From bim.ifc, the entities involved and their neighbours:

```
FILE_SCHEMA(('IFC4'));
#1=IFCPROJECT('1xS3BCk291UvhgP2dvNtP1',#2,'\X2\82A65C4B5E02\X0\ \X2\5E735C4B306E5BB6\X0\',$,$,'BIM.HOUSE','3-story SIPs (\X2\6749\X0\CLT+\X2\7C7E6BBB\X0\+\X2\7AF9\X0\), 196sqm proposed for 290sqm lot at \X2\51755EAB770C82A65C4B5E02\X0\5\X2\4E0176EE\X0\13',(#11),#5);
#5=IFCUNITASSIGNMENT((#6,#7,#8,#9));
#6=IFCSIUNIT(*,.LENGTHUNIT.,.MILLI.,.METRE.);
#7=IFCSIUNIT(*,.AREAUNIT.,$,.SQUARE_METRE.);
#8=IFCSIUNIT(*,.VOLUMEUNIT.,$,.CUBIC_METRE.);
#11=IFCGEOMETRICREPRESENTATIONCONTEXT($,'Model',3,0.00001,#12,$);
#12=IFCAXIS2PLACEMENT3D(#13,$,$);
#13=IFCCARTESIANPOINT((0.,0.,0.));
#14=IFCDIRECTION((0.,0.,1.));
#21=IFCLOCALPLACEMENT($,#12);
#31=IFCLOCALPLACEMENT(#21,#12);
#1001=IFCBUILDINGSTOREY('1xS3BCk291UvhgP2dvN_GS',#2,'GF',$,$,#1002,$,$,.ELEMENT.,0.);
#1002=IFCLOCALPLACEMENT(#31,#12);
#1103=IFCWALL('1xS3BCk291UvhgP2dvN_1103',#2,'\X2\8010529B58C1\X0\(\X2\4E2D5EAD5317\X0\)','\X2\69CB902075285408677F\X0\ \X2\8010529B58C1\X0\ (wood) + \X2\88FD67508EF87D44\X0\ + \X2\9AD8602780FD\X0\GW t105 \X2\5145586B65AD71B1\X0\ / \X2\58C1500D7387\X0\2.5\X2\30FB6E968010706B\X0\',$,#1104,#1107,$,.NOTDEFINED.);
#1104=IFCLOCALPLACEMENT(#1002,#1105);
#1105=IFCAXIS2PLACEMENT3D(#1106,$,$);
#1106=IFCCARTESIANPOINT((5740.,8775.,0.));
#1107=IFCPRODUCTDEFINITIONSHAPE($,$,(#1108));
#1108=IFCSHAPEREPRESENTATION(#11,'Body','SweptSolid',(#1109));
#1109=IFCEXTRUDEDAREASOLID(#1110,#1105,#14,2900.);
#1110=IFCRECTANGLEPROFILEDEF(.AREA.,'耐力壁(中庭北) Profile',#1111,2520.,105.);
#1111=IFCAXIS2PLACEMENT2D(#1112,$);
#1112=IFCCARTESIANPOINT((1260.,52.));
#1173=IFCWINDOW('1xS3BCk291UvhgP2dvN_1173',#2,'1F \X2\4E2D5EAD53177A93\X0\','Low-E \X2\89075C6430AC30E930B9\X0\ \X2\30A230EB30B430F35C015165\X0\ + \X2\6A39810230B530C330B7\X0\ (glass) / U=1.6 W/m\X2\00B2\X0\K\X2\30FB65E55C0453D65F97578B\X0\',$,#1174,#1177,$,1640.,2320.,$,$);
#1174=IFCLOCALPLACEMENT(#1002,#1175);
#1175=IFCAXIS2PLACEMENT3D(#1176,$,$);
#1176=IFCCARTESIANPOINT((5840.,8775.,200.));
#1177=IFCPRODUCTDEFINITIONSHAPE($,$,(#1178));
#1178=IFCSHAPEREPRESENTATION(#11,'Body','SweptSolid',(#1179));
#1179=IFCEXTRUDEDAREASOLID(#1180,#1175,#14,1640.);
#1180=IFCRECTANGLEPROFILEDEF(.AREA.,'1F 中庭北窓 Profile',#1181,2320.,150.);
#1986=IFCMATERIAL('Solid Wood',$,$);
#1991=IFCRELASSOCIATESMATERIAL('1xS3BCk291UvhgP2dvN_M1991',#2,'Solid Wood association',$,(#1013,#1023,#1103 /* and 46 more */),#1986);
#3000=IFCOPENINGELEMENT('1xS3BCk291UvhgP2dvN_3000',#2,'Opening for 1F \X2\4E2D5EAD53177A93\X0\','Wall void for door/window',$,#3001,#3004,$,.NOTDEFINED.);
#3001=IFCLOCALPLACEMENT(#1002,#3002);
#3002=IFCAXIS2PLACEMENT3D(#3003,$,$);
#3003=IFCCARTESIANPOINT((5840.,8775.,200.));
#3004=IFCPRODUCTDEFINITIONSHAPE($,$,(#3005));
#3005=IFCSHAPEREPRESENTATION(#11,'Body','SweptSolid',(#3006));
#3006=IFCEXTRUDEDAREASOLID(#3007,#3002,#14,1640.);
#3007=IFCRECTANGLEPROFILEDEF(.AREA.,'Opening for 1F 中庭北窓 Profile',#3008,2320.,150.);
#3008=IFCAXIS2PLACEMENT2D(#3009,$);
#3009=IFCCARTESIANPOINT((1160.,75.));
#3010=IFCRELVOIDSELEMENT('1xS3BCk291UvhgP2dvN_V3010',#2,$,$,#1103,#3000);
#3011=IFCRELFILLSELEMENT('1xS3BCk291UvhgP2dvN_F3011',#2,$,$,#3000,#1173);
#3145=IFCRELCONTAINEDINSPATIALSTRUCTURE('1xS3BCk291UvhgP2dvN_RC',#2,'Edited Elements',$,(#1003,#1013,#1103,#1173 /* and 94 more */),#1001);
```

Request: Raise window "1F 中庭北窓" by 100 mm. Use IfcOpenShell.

```python
import numpy as np
import ifcopenshell
import ifcopenshell.api.geometry
import ifcopenshell.util.placement
import ifcopenshell.util.unit

model = ifcopenshell.open("bim.ifc")
unit_scale = ifcopenshell.util.unit.calculate_unit_scale(model)

window = model.by_id(1173)
opening = window.FillsVoids[0].RelatingOpeningElement
dz = 100.0

shift = np.array([0.0, 0.0, dz])
# The window is not placed relative to its opening, so move both.
for product in (opening, window):
    matrix = ifcopenshell.util.placement.get_local_placement(product.ObjectPlacement)
    matrix[:3, 3] += shift
    ifcopenshell.api.geometry.edit_object_placement(model, product=product, matrix=matrix, is_si=False)

print(f"moved by {dz * unit_scale:+.3f} m")

model.write("bim_edited.ifc")
```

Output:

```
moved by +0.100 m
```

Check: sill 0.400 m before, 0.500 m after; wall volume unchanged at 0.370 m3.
